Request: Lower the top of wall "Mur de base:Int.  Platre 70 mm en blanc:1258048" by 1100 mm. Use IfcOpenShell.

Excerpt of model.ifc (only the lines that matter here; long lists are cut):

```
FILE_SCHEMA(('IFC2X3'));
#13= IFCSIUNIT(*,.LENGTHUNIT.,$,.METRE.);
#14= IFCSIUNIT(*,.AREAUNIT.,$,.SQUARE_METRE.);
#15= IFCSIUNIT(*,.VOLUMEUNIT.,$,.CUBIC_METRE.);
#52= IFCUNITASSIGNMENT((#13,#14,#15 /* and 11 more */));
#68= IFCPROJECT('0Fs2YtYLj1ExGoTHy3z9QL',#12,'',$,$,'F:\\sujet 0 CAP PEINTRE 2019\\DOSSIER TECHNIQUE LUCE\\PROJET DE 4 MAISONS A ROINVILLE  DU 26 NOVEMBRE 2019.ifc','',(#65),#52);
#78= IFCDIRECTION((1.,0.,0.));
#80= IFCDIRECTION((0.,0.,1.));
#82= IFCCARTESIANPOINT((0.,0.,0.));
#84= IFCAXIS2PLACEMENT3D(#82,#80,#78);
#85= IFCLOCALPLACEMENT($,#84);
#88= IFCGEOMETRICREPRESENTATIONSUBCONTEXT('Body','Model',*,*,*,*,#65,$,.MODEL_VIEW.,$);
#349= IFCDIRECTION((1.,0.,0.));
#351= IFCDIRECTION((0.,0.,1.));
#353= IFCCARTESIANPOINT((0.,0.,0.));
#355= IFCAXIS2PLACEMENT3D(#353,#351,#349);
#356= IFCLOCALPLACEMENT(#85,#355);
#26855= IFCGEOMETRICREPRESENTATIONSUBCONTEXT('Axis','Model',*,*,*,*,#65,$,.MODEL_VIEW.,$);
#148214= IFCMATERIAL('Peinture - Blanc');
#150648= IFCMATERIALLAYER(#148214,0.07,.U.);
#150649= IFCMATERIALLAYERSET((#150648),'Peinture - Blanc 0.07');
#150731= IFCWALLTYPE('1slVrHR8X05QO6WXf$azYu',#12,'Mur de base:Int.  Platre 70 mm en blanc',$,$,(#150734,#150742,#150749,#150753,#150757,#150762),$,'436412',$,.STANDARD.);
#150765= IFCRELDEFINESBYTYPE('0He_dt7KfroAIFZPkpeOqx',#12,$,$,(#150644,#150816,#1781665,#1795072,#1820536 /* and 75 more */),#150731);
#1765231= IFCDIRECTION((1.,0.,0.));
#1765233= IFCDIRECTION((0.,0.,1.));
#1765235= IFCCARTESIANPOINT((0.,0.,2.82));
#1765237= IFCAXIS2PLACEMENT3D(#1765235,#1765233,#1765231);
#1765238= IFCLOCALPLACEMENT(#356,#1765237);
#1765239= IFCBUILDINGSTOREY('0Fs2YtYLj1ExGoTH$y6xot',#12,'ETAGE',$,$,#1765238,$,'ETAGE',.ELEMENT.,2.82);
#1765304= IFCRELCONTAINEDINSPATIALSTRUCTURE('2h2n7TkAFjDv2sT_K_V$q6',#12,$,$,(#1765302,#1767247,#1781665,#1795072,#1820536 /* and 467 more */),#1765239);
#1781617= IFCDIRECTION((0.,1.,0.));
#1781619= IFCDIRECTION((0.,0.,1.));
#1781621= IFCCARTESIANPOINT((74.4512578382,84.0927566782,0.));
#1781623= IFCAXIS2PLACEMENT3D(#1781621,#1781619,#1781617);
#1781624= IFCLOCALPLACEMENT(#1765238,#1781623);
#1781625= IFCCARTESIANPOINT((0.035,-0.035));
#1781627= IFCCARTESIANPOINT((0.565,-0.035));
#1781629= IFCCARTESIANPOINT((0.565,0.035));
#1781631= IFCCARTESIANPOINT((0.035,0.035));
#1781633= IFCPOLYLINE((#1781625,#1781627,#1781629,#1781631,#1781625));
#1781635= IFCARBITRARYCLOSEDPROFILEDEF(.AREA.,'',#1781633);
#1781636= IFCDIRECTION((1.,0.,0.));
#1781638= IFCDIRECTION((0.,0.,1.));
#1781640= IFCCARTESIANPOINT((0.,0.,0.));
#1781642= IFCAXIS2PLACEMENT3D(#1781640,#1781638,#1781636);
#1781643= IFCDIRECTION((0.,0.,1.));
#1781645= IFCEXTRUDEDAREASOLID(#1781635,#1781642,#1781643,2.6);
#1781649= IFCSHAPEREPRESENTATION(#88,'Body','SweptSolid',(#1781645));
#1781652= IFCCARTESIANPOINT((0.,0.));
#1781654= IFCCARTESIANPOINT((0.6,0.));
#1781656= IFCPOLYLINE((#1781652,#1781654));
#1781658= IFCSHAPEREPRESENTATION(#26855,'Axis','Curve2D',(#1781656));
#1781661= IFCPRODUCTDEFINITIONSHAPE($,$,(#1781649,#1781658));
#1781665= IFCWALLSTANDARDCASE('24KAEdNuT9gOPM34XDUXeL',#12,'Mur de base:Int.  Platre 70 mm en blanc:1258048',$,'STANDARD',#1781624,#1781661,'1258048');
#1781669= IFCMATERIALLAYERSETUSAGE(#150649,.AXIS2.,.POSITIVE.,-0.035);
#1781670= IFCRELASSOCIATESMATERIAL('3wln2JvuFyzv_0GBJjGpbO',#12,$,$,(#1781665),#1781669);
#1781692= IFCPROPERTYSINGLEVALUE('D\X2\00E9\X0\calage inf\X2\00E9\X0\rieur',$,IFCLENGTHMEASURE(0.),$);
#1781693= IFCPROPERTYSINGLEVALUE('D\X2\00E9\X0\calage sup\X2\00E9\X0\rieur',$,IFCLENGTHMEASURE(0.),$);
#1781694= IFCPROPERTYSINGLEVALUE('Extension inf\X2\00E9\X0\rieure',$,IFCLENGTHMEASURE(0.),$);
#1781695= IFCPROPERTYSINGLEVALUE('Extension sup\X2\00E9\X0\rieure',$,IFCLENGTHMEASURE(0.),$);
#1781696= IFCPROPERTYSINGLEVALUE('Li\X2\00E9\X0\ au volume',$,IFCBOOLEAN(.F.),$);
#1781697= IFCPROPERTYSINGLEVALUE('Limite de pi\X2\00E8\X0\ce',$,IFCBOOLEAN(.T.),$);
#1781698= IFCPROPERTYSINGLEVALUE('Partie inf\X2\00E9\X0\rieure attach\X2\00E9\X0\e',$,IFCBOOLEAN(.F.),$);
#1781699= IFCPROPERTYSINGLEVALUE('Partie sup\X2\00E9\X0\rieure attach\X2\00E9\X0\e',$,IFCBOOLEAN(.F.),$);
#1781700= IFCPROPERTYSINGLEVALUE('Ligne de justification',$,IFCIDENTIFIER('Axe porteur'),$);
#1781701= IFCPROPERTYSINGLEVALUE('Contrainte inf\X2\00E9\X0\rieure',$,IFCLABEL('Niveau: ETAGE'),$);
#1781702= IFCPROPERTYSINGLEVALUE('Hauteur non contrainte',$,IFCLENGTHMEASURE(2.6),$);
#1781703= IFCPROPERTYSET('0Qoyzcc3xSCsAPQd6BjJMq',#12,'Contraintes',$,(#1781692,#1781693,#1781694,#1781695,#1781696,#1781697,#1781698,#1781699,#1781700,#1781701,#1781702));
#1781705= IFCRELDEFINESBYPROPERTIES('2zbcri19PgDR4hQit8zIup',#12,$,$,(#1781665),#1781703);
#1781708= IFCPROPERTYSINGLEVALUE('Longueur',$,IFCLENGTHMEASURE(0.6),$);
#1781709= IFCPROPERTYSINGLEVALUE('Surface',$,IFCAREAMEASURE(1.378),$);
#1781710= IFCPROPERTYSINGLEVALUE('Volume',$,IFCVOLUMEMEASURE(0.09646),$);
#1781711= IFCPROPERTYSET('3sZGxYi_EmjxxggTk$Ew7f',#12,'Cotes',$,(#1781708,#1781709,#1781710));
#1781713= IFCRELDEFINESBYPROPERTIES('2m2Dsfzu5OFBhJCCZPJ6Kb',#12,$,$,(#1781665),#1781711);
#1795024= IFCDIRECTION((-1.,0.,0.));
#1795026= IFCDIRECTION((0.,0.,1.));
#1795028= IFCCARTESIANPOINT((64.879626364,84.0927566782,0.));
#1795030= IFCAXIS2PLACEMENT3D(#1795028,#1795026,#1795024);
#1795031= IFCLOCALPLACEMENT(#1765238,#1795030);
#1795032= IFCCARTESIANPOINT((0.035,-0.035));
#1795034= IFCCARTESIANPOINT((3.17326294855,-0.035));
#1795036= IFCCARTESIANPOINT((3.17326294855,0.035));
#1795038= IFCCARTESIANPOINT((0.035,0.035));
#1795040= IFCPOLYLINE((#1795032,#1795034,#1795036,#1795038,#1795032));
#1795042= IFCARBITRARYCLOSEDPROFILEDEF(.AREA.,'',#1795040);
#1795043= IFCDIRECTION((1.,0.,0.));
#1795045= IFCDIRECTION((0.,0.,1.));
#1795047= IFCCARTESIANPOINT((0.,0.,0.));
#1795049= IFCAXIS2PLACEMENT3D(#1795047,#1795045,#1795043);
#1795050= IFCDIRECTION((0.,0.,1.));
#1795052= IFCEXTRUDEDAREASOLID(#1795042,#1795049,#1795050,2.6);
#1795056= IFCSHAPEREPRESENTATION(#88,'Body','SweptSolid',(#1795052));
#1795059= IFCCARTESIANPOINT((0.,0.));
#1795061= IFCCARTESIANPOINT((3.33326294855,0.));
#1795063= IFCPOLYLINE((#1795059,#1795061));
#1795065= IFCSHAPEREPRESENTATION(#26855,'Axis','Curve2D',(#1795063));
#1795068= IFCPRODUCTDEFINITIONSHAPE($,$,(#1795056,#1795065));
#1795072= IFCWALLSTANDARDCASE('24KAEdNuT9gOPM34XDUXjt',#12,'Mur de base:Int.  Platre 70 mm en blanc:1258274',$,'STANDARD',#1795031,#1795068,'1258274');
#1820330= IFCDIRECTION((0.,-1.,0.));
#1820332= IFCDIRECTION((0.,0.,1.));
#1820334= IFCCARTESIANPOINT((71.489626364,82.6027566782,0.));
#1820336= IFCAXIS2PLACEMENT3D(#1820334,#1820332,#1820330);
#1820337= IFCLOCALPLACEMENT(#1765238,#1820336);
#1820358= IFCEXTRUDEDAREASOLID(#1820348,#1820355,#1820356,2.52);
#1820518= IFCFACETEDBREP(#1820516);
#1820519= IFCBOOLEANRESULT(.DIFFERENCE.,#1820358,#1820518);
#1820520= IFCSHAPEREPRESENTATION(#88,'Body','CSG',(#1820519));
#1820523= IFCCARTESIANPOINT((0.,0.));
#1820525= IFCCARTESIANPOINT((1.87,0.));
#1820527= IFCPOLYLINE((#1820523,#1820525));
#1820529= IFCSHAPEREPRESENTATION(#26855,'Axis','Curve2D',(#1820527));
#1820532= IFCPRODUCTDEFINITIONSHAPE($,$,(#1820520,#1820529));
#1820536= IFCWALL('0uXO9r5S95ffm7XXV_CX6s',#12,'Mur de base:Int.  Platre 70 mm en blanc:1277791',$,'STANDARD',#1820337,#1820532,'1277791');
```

```python
import ifcopenshell
import ifcopenshell.api.pset
import ifcopenshell.geom
import ifcopenshell.util.element
import ifcopenshell.util.representation
import ifcopenshell.util.shape
import ifcopenshell.util.unit

model = ifcopenshell.open("model.ifc")
area_scale = ifcopenshell.util.unit.calculate_unit_scale(model, "AREAUNIT")
volume_scale = ifcopenshell.util.unit.calculate_unit_scale(model, "VOLUMEUNIT")
settings = ifcopenshell.geom.settings()


def volume(element):
    """Net volume in cubic metres, openings subtracted."""
    shape = ifcopenshell.geom.create_shape(settings, element)
    return ifcopenshell.util.shape.get_volume(shape.geometry)


wall = model.by_guid("24KAEdNuT9gOPM34XDUXeL")
before = volume(wall)

body = ifcopenshell.util.representation.get_representation(wall, "Model", "Body")
solid = body.Items[0]
old_height = solid.Depth
solid.Depth -= 1.1
after = volume(wall)
thickness = 0.07  # wall thickness in metres

# Update the stored height, areas and volumes.
pset = model.by_id(ifcopenshell.util.element.get_pset(wall, "Contraintes", should_inherit=False)["id"])
ifcopenshell.api.pset.edit_pset(model, pset=pset, properties={
    "Hauteur non contrainte": model.create_entity("IfcLengthMeasure", solid.Depth),
})
pset = model.by_id(ifcopenshell.util.element.get_pset(wall, "Cotes", should_inherit=False)["id"])
ifcopenshell.api.pset.edit_pset(model, pset=pset, properties={
    "Surface": model.create_entity("IfcAreaMeasure", after / thickness / area_scale),
    "Volume": model.create_entity("IfcVolumeMeasure", after / volume_scale),
})

print(f"height {old_height:g} -> {solid.Depth:g}, volume {before:.3f} -> {after:.3f} m3")

model.write("model_rev.ifc")
```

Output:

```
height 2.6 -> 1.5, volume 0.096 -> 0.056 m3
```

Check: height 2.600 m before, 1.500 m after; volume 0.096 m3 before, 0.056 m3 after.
